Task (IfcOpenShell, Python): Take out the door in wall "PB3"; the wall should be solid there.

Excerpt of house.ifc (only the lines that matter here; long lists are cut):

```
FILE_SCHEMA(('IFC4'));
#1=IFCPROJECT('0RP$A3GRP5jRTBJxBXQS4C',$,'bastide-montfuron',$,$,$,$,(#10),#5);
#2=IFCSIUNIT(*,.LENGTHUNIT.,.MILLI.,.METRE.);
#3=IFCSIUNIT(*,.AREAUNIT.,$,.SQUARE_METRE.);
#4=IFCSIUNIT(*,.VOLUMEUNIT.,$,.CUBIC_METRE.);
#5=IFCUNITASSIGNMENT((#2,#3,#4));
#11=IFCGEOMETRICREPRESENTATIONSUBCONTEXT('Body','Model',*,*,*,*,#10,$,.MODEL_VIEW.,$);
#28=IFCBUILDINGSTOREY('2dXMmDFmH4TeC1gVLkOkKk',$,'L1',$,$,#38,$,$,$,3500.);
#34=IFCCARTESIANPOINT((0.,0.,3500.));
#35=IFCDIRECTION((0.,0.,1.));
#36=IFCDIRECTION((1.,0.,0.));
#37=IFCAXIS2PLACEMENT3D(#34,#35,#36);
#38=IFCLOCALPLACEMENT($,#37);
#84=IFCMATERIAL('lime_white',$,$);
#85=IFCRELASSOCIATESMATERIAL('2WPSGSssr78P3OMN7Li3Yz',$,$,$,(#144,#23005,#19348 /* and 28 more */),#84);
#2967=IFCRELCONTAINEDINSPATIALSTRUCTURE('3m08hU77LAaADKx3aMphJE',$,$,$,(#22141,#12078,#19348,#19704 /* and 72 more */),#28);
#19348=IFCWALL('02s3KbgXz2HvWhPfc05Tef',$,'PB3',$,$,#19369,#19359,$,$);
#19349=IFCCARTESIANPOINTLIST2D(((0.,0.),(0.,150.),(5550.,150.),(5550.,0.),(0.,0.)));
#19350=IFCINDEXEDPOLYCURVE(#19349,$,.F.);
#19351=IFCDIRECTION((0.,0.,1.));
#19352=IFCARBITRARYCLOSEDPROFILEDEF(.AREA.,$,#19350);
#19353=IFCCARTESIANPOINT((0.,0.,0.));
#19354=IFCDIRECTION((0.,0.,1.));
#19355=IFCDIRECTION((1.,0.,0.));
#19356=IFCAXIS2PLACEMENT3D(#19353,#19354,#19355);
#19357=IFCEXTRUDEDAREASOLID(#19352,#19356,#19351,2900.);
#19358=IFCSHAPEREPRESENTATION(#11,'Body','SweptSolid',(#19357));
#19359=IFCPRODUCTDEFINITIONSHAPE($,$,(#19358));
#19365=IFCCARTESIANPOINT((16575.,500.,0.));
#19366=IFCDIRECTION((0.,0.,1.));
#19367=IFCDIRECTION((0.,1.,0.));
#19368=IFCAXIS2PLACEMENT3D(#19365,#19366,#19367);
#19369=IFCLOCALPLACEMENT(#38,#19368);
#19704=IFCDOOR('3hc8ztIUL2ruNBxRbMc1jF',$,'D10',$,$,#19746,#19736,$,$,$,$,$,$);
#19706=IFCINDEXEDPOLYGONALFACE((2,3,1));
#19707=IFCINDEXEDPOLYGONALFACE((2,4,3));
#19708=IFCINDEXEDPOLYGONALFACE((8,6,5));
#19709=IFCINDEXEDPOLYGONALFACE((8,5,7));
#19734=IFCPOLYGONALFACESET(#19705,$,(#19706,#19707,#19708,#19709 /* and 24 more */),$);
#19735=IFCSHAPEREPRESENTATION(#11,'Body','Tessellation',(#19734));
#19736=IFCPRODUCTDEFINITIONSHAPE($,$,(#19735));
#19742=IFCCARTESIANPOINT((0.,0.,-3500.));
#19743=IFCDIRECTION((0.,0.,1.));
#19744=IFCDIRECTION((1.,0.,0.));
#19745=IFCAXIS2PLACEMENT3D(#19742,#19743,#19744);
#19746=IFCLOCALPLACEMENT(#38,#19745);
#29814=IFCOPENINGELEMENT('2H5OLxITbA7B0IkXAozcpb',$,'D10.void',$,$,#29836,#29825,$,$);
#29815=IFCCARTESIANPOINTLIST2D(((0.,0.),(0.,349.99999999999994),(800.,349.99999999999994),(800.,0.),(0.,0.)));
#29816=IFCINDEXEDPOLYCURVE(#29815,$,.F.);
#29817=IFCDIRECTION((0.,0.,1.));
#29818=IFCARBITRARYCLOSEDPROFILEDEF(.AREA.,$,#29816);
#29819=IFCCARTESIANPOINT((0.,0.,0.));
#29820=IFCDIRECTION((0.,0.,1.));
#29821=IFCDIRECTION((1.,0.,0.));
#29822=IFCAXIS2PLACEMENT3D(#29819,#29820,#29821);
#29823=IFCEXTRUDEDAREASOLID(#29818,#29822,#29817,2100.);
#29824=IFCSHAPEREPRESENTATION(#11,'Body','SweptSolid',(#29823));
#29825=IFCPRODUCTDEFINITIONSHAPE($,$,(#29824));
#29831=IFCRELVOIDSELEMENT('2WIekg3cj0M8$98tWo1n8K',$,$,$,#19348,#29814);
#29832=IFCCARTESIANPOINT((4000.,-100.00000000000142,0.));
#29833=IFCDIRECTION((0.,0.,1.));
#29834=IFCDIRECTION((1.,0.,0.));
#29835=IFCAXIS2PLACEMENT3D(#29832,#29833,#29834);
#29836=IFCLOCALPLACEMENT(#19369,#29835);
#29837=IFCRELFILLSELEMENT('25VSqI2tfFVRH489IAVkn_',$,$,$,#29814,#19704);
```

```python
import ifcopenshell
import ifcopenshell.api.feature
import ifcopenshell.api.root
import ifcopenshell.geom
import ifcopenshell.util.shape

model = ifcopenshell.open("house.ifc")
settings = ifcopenshell.geom.settings()


def volume(element):
    """Net volume in cubic metres, openings subtracted."""
    shape = ifcopenshell.geom.create_shape(settings, element)
    return ifcopenshell.util.shape.get_volume(shape.geometry)


door = model.by_id(19704)
opening = door.FillsVoids[0].RelatingOpeningElement
wall = opening.VoidsElements[0].RelatingBuildingElement
before = volume(wall)

ifcopenshell.api.root.remove_product(model, product=door)
ifcopenshell.api.feature.remove_feature(model, feature=opening)

after = volume(wall)

print(f"wall volume {before:.3f} -> {after:.3f} m3")

model.write("house-out.ifc")
```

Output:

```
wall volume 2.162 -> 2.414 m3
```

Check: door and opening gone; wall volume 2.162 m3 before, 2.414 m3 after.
